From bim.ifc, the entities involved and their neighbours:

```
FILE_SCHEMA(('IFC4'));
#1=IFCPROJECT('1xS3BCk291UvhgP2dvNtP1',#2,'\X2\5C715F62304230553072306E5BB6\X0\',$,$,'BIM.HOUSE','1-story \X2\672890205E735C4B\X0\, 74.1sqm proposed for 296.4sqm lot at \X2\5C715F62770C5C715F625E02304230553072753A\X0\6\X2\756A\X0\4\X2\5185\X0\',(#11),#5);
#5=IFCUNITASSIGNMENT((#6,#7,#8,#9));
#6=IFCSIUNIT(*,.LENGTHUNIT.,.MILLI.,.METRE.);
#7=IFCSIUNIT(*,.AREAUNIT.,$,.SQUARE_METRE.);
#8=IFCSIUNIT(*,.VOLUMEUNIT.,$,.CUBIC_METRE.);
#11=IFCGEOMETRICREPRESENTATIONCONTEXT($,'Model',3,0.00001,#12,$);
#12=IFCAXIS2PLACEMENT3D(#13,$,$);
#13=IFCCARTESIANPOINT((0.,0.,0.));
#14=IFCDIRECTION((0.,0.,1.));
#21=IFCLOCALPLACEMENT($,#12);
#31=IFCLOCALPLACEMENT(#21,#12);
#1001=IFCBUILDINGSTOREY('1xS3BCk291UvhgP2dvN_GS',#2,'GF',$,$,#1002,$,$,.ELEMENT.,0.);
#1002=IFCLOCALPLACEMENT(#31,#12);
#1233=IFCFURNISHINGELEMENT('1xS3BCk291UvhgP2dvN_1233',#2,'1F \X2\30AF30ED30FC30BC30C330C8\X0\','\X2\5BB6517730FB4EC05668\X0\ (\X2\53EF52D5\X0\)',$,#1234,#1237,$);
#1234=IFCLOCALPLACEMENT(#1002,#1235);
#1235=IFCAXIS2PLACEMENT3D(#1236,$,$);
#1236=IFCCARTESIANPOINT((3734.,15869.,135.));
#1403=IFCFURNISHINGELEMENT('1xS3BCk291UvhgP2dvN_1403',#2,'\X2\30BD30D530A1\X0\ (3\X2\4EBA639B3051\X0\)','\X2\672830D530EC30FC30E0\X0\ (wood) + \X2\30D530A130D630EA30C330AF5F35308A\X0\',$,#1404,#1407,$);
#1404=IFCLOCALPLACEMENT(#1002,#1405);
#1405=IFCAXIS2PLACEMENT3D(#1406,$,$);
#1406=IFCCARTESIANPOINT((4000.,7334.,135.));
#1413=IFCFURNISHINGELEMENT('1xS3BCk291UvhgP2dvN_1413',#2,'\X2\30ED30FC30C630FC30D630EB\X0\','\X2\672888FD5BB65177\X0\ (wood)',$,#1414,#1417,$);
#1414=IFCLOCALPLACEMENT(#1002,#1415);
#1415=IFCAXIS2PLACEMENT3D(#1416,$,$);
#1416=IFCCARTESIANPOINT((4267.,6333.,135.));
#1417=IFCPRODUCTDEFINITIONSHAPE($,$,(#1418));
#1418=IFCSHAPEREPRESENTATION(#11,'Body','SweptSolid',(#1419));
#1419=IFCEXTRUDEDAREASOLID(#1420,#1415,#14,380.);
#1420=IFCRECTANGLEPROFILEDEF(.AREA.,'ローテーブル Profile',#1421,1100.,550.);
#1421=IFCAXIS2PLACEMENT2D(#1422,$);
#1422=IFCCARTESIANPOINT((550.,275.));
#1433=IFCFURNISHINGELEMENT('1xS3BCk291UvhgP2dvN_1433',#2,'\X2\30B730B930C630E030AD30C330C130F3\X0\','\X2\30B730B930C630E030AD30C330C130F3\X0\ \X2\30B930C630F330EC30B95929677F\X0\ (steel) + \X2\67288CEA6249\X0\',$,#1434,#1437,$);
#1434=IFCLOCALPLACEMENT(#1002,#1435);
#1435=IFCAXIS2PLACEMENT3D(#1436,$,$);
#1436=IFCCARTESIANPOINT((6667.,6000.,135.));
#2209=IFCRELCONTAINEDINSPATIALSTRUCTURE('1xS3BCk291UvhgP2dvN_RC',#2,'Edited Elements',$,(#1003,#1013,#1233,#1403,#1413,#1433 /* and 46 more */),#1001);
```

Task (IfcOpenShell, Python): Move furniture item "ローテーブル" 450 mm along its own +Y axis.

```python
import ifcopenshell
import ifcopenshell.api.geometry
import ifcopenshell.util.placement
import ifcopenshell.util.unit

model = ifcopenshell.open("bim.ifc")
unit_scale = ifcopenshell.util.unit.calculate_unit_scale(model)

item = model.by_id(1413)
matrix = ifcopenshell.util.placement.get_local_placement(item.ObjectPlacement)
matrix[:3, 3] += matrix[:3, 1] * 0.45 / unit_scale
ifcopenshell.api.geometry.edit_object_placement(model, product=item, matrix=matrix, is_si=False)

print(ifcopenshell.util.placement.get_local_placement(item.ObjectPlacement).round(3) + 0.0)

model.write("bim_updated.ifc")
```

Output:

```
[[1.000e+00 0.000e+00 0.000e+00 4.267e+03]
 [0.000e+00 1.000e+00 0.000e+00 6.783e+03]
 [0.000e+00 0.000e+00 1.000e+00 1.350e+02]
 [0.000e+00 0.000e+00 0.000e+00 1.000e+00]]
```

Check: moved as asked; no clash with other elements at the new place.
